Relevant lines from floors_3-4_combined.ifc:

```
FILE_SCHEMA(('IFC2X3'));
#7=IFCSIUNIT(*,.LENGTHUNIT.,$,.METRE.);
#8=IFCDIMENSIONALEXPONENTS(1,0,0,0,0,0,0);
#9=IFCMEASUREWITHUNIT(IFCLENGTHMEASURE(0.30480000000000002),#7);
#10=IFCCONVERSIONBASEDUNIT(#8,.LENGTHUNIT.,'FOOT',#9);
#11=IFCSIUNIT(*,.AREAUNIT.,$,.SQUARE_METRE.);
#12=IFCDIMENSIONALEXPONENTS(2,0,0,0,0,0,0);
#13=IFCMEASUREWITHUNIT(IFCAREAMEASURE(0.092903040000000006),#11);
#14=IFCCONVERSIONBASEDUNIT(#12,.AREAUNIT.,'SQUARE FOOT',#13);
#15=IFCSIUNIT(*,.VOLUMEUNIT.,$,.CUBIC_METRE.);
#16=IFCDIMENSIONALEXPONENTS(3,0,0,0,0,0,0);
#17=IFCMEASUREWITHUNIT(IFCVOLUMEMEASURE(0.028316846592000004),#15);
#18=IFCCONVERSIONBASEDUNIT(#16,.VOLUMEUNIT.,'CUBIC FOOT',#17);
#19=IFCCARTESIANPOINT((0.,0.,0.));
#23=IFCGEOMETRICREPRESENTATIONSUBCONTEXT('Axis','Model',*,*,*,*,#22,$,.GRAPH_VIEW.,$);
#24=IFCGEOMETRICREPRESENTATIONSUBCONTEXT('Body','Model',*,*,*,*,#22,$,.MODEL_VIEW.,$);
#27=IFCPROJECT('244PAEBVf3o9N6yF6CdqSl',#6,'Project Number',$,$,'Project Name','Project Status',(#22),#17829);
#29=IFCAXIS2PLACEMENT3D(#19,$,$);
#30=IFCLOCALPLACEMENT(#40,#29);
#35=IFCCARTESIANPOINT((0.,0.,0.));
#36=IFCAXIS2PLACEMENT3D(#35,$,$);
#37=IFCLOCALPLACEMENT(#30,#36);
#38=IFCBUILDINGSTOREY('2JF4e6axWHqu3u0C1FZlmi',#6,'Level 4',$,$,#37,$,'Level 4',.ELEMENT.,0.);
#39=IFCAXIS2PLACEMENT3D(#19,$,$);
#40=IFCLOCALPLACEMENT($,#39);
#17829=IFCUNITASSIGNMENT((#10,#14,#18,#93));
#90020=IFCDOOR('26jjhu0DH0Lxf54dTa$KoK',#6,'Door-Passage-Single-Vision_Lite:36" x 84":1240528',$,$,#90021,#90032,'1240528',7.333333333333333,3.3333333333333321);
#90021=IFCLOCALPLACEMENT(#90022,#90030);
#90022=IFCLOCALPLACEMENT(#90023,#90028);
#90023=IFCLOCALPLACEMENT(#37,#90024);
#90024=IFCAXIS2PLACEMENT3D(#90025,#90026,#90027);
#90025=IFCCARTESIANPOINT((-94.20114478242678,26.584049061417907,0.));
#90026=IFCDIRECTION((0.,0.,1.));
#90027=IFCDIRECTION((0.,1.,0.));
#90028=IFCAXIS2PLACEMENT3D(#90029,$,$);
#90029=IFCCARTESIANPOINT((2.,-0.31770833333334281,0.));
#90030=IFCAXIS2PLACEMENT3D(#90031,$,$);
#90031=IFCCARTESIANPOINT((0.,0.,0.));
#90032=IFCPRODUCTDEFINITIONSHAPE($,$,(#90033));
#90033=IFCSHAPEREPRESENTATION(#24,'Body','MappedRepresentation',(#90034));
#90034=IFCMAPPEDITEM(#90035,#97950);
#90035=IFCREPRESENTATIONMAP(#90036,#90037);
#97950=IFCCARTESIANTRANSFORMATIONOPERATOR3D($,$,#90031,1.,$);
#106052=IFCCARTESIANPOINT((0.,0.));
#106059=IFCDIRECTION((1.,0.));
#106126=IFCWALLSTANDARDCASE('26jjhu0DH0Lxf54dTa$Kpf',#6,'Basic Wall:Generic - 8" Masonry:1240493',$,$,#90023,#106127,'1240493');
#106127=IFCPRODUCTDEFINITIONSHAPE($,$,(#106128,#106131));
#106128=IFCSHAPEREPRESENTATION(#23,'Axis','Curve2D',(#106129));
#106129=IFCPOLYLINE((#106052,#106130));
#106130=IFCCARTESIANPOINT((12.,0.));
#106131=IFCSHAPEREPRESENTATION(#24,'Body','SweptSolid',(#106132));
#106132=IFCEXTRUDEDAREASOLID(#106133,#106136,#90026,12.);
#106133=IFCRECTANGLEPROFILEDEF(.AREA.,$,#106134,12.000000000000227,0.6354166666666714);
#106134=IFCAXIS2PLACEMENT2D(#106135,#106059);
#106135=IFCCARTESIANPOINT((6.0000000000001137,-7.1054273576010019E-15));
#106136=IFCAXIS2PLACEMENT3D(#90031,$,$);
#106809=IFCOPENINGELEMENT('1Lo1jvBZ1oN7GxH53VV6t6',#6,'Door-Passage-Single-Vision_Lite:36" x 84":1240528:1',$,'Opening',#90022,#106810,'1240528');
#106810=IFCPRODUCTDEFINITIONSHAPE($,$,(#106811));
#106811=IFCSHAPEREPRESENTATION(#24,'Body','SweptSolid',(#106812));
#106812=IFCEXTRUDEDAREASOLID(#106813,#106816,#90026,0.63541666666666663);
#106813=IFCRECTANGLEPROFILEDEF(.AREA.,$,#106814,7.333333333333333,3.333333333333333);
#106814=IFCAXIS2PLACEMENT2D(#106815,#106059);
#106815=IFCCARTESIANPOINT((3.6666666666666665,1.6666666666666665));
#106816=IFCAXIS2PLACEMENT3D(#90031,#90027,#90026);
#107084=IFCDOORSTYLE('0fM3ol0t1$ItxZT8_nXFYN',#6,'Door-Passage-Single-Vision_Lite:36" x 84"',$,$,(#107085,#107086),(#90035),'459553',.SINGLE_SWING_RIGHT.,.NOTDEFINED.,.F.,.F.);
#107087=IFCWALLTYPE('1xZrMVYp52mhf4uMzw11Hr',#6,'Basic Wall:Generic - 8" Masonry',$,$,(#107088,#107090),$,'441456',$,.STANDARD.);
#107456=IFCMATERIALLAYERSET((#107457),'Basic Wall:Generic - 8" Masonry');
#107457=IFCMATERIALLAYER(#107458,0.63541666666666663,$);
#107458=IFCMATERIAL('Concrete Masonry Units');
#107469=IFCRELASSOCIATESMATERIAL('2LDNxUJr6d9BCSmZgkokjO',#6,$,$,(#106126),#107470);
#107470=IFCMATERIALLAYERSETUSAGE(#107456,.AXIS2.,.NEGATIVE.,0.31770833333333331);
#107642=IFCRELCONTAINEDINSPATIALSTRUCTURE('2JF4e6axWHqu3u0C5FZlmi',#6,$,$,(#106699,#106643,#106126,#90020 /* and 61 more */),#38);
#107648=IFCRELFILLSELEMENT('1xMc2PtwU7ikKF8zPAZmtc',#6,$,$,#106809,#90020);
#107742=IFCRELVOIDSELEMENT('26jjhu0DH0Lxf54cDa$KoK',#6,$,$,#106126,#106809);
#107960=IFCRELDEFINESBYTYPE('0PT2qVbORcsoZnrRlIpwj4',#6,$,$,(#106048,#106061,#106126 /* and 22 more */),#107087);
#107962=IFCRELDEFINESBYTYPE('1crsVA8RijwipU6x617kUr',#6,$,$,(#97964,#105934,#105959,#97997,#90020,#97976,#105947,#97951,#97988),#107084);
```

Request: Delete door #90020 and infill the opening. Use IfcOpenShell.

```python
import ifcopenshell
import ifcopenshell.api.feature
import ifcopenshell.api.root
import ifcopenshell.geom
import ifcopenshell.util.shape

model = ifcopenshell.open("floors_3-4_combined.ifc")
settings = ifcopenshell.geom.settings()


def volume(element):
    """Net volume in cubic metres, openings subtracted."""
    shape = ifcopenshell.geom.create_shape(settings, element)
    return ifcopenshell.util.shape.get_volume(shape.geometry)


door = model.by_id(90020)
opening = door.FillsVoids[0].RelatingOpeningElement
wall = opening.VoidsElements[0].RelatingBuildingElement
before = volume(wall)

ifcopenshell.api.root.remove_product(model, product=door)
ifcopenshell.api.feature.remove_feature(model, feature=opening)

after = volume(wall)

print(f"wall volume {before:.3f} -> {after:.3f} m3")

model.write("floors_3-4_combined_v2.ifc")
```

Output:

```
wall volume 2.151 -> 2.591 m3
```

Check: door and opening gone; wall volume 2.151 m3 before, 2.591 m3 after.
